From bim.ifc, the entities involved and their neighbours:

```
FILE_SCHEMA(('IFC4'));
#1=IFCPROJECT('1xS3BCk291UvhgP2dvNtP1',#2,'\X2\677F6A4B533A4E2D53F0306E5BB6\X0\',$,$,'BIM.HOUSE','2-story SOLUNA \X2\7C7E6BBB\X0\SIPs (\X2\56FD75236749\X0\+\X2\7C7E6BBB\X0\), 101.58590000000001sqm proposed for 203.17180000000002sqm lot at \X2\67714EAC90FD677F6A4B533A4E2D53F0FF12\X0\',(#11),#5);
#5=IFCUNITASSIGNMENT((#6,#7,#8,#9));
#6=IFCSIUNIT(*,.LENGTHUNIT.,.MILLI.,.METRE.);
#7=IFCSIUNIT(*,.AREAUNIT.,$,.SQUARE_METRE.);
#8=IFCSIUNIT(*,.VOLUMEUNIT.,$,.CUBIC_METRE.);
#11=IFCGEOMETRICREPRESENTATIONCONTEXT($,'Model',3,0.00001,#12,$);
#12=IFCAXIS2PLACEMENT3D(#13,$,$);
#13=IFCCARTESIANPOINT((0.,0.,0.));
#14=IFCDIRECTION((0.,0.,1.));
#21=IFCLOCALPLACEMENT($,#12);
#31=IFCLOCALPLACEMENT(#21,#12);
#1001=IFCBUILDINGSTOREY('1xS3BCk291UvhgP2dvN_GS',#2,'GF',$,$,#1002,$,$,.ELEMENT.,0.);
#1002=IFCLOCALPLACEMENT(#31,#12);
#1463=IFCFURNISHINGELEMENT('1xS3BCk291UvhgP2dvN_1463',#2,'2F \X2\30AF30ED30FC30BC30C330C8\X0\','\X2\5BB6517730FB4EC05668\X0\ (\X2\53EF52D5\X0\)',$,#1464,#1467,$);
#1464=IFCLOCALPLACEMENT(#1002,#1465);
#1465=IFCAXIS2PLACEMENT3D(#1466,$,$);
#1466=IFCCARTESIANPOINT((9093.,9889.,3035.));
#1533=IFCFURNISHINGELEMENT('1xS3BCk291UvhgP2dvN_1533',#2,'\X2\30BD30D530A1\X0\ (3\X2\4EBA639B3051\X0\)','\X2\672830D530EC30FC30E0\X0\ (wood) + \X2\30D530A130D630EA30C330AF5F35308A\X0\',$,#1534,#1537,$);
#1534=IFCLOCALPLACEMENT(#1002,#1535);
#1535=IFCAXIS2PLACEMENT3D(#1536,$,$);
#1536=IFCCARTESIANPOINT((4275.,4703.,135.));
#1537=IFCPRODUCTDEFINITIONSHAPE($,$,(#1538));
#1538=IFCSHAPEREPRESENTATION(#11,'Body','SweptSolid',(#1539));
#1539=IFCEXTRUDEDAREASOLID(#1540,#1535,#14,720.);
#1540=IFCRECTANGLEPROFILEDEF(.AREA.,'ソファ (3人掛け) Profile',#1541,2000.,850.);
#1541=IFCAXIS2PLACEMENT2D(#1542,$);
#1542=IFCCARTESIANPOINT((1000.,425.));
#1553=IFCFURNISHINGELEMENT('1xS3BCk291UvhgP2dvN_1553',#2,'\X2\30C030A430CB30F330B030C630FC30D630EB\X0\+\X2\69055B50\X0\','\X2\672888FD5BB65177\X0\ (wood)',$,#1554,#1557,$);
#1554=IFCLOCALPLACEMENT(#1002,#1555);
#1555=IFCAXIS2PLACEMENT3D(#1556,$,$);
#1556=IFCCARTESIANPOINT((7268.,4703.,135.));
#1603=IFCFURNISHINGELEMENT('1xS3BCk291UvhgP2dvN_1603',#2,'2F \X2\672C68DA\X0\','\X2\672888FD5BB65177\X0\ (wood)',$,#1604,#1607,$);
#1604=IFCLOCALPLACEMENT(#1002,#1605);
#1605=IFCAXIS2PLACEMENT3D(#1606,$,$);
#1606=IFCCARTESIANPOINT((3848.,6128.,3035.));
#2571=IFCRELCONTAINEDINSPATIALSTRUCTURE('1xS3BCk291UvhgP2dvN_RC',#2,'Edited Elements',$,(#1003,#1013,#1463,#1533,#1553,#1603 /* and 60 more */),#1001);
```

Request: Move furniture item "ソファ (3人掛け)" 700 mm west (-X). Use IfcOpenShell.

```python
import ifcopenshell
import ifcopenshell.api.geometry
import ifcopenshell.util.placement
import ifcopenshell.util.unit

model = ifcopenshell.open("bim.ifc")
unit_scale = ifcopenshell.util.unit.calculate_unit_scale(model)

item = model.by_guid("1xS3BCk291UvhgP2dvN_1533")
matrix = ifcopenshell.util.placement.get_local_placement(item.ObjectPlacement)
matrix[0, 3] -= 0.7 / unit_scale
ifcopenshell.api.geometry.edit_object_placement(model, product=item, matrix=matrix, is_si=False)

print(ifcopenshell.util.placement.get_local_placement(item.ObjectPlacement).round(3) + 0.0)

model.write("bim_updated.ifc")
```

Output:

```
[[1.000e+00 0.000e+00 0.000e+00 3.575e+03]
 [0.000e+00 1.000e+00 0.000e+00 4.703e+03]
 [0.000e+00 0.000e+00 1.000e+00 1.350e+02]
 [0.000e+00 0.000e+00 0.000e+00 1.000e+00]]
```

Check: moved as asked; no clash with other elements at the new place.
